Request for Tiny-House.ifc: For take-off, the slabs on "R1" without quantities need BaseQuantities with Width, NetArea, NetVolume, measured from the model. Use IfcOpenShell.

First a look at what the model holds.

```python
import ifcopenshell
import ifcopenshell.util.element
import ifcopenshell.util.unit

model = ifcopenshell.open("Tiny-House.ifc")
print(model.schema)
for unit_type in ("LENGTHUNIT", "AREAUNIT", "VOLUMEUNIT"):
    print(unit_type, ifcopenshell.util.unit.calculate_unit_scale(model, unit_type))
storey = next(s for s in model.by_type("IfcBuildingStorey") if s.Name == "R1")
slabs = [e for e in ifcopenshell.util.element.get_decomposition(storey) if e.is_a("IfcSlab")]
for e in sorted(slabs, key=lambda e: e.id()):
    print(e.id(), e.is_a(), e.Name, list(ifcopenshell.util.element.get_psets(e, qtos_only=True)), sep=" | ")
```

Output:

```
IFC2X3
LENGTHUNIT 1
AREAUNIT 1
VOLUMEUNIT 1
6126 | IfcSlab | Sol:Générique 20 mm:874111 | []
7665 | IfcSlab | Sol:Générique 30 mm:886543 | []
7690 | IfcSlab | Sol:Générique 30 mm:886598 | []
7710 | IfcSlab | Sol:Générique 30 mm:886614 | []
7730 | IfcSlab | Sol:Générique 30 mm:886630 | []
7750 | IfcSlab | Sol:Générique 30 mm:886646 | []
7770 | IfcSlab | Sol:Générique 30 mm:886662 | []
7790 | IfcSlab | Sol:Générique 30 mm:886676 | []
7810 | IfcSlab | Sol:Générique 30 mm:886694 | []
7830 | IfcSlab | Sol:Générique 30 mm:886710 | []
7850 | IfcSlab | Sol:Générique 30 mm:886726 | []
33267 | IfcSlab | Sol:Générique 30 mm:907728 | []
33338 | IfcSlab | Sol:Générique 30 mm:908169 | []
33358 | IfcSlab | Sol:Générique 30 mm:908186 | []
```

```python
import ifcopenshell
import ifcopenshell.api.pset
import ifcopenshell.geom
import ifcopenshell.util.element
import ifcopenshell.util.shape
import ifcopenshell.util.unit

model = ifcopenshell.open("Tiny-House.ifc")
unit_scale = ifcopenshell.util.unit.calculate_unit_scale(model)
area_scale = ifcopenshell.util.unit.calculate_unit_scale(model, "AREAUNIT")
volume_scale = ifcopenshell.util.unit.calculate_unit_scale(model, "VOLUMEUNIT")
settings = ifcopenshell.geom.settings()

storey = next(s for s in model.by_type("IfcBuildingStorey") if s.Name == "R1")
slabs = [e for e in ifcopenshell.util.element.get_decomposition(storey) if e.is_a("IfcSlab")]

for e in sorted(slabs, key=lambda e: e.id()):
    if ifcopenshell.util.element.get_psets(e, qtos_only=True, should_inherit=False):
        continue
    # Geometry comes back in metres, in the element's own axes.
    shape = ifcopenshell.geom.create_shape(settings, e)
    values = {
        "Width": ifcopenshell.util.shape.get_z(shape.geometry) / unit_scale,
        "NetArea": ifcopenshell.util.shape.get_footprint_area(shape.geometry) / area_scale,
        "NetVolume": ifcopenshell.util.shape.get_volume(shape.geometry) / volume_scale,
    }
    qto = ifcopenshell.api.pset.add_qto(model, product=e, name="BaseQuantities")
    ifcopenshell.api.pset.edit_qto(model, qto=qto, properties=values)
    print(e.id(), {k: round(v, 3) for k, v in values.items()})

model.write("Tiny-House_edited.ifc")
```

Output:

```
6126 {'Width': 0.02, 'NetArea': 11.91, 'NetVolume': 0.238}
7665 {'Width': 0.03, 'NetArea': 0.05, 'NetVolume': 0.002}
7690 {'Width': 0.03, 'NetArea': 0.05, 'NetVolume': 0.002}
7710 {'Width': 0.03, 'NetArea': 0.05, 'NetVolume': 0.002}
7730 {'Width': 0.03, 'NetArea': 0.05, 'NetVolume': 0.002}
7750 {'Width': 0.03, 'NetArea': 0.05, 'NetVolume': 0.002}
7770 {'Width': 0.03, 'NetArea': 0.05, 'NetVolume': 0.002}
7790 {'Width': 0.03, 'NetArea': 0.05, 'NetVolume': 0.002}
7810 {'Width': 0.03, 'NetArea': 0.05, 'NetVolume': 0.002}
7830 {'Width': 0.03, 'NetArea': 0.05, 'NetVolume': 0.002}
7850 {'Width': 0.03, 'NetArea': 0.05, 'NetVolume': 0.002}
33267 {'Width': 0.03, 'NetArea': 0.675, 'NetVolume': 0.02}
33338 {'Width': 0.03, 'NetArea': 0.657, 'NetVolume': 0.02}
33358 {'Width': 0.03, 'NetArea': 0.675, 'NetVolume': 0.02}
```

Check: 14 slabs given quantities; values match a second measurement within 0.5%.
